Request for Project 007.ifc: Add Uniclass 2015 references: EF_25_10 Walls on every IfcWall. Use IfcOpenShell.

First a look at what the model holds.

```python
import ifcopenshell

model = ifcopenshell.open("Project 007.ifc")
print(model.schema)
print("classifications:", [c.Name for c in model.by_type("IfcClassification")])
for ifc_class in ("IfcDoor", "IfcRoof", "IfcStair", "IfcWall", "IfcWindow"):
    print(ifc_class, len(model.by_type(ifc_class)))
```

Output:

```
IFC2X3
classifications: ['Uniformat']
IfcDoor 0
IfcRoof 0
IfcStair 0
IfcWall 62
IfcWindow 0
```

```python
import ifcopenshell
import ifcopenshell.api.classification

model = ifcopenshell.open("Project 007.ifc")

# IFC2X3 requires Source and Edition and has no link from the project to the system.
system = model.create_entity("IfcClassification", Source="NBS", Edition="2015", Name="Uniclass 2015")

codes = {
    "IfcWall": ("EF_25_10", "Walls"),
}
for ifc_class, (code, name) in codes.items():
    products = model.by_type(ifc_class)
    ifcopenshell.api.classification.add_reference(
        model, products=products, classification=system, identification=code, name=name
    )
    print(code, len(products))

model.write("Project 007_rev.ifc")
```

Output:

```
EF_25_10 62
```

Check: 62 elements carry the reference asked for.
